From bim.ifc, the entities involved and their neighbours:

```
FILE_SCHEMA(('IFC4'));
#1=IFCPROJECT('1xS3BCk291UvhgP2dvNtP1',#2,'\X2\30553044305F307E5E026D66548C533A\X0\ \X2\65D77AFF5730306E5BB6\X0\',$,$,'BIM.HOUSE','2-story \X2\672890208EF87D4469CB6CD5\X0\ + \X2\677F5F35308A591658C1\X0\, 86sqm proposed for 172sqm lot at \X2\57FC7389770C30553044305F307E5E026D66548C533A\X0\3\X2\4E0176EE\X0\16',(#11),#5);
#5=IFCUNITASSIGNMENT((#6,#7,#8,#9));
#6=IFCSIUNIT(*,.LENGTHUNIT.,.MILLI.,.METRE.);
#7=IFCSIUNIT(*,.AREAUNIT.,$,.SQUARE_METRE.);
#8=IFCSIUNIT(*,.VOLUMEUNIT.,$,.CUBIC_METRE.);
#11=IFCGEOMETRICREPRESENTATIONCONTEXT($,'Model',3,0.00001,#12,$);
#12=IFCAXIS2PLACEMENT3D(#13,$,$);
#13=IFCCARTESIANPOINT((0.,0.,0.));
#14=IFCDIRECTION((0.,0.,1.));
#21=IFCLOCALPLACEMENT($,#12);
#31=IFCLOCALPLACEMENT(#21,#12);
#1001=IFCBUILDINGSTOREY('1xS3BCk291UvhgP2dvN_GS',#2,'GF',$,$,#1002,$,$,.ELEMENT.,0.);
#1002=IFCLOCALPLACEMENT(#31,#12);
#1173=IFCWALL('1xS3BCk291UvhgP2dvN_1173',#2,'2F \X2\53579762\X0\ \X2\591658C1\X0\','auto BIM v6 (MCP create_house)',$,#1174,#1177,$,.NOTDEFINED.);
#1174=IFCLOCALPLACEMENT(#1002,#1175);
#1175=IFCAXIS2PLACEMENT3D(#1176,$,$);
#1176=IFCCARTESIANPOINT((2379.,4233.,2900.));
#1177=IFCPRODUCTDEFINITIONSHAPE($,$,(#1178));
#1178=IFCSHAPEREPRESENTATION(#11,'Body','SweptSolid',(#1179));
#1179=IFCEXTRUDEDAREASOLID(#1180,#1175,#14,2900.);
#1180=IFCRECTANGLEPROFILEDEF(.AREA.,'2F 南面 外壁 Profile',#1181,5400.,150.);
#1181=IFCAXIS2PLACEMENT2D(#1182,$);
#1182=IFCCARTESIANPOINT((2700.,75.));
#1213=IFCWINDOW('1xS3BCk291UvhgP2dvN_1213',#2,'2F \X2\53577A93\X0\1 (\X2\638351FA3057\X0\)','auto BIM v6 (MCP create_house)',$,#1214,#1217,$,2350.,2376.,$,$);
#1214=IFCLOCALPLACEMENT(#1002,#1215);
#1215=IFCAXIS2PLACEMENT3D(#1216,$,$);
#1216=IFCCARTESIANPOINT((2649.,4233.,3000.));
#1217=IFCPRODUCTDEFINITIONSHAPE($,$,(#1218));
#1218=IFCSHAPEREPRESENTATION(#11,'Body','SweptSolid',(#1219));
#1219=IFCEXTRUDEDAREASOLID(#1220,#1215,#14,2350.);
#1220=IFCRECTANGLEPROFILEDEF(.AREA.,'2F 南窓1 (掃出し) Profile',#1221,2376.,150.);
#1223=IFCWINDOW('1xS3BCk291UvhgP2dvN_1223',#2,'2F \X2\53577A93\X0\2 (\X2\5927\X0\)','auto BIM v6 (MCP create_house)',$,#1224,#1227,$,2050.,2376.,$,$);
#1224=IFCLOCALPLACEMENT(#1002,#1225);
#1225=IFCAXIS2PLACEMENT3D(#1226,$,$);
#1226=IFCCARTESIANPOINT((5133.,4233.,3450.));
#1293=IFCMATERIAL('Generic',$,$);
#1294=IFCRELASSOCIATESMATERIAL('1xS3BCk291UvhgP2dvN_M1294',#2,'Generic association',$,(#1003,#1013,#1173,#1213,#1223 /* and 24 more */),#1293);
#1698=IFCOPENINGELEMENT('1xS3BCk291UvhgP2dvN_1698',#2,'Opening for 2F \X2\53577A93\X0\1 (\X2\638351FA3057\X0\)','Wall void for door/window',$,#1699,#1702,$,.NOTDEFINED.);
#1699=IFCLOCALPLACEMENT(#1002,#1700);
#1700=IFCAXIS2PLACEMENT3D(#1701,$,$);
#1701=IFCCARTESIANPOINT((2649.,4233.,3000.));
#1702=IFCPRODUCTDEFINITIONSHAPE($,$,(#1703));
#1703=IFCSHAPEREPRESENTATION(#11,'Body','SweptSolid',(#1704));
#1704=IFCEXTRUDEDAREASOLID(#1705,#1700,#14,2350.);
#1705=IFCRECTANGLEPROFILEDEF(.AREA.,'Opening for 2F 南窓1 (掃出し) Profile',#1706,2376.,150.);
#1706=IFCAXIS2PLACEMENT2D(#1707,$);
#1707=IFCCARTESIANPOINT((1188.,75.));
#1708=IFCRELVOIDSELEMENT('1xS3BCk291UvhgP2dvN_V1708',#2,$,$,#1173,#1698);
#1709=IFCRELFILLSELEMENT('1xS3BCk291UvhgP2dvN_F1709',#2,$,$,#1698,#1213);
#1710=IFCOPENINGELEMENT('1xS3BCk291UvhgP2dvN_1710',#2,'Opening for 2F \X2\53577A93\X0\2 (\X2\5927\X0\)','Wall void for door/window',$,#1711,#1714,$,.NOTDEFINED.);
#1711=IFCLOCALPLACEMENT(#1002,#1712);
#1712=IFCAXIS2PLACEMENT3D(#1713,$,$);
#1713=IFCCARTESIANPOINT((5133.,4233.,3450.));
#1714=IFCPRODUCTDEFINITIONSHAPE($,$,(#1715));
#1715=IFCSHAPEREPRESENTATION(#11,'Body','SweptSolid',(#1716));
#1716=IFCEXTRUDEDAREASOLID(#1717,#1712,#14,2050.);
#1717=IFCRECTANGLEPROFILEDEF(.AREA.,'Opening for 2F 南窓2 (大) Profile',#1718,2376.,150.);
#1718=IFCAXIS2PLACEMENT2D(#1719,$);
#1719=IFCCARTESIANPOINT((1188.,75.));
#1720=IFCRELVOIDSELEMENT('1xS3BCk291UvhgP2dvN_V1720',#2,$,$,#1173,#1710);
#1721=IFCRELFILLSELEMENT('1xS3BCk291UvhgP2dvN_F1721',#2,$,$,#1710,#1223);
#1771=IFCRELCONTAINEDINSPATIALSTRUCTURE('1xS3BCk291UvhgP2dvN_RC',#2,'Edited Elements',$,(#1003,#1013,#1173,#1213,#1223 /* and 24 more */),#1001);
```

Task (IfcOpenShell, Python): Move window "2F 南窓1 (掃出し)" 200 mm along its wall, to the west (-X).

```python
import ifcopenshell
import ifcopenshell.api.geometry
import ifcopenshell.util.placement
import ifcopenshell.util.unit

model = ifcopenshell.open("bim.ifc")
unit_scale = ifcopenshell.util.unit.calculate_unit_scale(model)

window = model.by_guid("1xS3BCk291UvhgP2dvN_1213")
opening = window.FillsVoids[0].RelatingOpeningElement
wall = opening.VoidsElements[0].RelatingBuildingElement

wall_matrix = ifcopenshell.util.placement.get_local_placement(wall.ObjectPlacement)
shift = wall_matrix[:3, 0] * -0.2 / unit_scale
before = ifcopenshell.util.placement.get_local_placement(window.ObjectPlacement)[:3, 3].copy()

# The window is not placed relative to its opening, so move both.
for product in (opening, window):
    matrix = ifcopenshell.util.placement.get_local_placement(product.ObjectPlacement)
    matrix[:3, 3] += shift
    ifcopenshell.api.geometry.edit_object_placement(model, product=product, matrix=matrix, is_si=False)

after = ifcopenshell.util.placement.get_local_placement(window.ObjectPlacement)[:3, 3]
print("window moved by", (after - before).round(3) + 0.0)

model.write("bim_v2.ifc")
```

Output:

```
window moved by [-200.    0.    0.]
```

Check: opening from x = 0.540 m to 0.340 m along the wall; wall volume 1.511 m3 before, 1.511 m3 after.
